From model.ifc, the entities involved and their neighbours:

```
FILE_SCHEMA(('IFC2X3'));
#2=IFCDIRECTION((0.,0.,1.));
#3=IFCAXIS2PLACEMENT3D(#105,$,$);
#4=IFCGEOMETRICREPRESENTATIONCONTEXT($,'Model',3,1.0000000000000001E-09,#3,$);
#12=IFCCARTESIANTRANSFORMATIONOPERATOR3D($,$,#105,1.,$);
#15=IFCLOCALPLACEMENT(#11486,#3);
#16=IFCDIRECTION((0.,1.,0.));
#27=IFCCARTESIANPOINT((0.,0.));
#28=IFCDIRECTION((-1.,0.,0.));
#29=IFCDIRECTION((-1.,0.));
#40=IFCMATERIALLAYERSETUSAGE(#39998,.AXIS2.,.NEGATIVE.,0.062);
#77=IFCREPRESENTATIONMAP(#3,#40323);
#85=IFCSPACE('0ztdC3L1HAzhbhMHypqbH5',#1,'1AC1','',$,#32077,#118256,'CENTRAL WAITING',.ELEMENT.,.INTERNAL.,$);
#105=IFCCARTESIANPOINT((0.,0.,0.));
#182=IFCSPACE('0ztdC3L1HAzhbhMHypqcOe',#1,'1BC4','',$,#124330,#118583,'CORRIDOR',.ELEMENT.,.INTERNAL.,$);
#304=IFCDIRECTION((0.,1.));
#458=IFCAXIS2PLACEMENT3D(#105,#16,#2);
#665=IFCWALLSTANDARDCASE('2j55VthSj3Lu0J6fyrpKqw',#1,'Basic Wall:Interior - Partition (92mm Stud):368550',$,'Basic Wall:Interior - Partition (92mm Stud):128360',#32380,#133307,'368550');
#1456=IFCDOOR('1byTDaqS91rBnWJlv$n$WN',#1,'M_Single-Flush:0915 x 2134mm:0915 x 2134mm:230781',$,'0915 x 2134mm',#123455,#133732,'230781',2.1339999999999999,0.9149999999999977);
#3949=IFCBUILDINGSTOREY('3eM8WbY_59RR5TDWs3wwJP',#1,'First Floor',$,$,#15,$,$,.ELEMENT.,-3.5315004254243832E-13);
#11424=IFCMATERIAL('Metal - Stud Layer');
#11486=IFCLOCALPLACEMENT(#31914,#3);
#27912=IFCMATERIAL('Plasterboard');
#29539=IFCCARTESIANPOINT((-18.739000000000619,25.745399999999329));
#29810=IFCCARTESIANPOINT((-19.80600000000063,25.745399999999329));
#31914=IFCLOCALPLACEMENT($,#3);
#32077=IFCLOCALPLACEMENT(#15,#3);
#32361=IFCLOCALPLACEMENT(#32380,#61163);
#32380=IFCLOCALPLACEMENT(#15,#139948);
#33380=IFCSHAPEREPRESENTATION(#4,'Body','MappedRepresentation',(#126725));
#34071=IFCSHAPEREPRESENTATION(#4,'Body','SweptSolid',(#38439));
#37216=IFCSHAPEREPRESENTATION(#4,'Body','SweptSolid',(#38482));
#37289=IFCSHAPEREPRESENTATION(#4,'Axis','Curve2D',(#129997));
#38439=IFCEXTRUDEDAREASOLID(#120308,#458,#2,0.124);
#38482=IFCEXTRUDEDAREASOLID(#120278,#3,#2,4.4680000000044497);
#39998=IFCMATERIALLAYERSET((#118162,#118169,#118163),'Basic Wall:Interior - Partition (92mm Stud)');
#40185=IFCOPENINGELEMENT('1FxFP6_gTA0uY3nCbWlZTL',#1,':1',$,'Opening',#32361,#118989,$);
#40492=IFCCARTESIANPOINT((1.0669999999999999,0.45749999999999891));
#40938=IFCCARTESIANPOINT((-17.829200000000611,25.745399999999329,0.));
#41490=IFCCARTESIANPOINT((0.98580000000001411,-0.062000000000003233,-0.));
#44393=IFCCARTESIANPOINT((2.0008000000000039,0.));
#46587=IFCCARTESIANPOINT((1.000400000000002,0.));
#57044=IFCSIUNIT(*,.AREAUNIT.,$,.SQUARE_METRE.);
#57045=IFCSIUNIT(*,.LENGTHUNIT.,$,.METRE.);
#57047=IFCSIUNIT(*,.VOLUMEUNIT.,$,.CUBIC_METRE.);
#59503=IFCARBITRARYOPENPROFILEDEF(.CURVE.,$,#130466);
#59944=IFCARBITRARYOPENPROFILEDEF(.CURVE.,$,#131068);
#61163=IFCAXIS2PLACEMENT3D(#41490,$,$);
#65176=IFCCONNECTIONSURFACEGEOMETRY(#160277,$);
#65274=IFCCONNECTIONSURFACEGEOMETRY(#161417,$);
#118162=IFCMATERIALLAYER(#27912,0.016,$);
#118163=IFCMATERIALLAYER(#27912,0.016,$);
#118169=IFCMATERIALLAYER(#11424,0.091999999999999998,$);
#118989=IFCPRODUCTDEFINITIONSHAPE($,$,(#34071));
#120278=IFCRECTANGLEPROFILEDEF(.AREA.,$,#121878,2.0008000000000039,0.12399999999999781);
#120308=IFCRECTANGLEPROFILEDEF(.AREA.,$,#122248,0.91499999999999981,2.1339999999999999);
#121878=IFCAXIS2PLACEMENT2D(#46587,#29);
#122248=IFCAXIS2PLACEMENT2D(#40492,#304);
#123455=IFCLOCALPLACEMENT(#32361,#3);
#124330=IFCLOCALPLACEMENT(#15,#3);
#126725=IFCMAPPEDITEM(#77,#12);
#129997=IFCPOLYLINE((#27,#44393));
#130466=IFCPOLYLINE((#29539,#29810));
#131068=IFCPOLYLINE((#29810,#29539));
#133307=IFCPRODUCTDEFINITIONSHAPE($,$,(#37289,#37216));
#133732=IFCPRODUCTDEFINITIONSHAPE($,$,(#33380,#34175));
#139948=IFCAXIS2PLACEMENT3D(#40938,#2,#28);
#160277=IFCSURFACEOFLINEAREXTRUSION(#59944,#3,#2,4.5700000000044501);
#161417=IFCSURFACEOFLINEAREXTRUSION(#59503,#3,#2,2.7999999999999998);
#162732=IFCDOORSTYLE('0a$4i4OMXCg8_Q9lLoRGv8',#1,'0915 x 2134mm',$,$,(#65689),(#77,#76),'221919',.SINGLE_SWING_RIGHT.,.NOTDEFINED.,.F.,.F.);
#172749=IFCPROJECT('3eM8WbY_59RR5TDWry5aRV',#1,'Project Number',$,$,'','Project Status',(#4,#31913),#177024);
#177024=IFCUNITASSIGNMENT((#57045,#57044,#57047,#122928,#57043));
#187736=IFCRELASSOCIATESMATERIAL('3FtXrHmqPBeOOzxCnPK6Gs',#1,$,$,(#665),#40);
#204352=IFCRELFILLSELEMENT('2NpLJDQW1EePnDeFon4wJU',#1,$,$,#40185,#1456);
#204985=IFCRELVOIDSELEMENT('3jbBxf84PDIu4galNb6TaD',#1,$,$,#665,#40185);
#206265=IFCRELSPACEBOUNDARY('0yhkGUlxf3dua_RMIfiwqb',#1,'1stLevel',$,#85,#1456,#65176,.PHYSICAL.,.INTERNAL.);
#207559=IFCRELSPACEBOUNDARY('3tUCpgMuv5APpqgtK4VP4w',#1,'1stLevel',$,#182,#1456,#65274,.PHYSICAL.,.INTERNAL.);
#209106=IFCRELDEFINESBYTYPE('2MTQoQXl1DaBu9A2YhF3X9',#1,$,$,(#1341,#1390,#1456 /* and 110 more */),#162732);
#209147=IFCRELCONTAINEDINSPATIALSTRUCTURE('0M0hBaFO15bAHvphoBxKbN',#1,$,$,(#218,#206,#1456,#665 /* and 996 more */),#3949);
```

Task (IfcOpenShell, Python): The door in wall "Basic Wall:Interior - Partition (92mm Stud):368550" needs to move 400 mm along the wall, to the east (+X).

```python
import numpy as np
import ifcopenshell
import ifcopenshell.api.geometry
import ifcopenshell.util.placement
import ifcopenshell.util.unit

model = ifcopenshell.open("model.ifc")
unit_scale = ifcopenshell.util.unit.calculate_unit_scale(model)

door = model.by_guid("1byTDaqS91rBnWJlv$n$WN")
opening = door.FillsVoids[0].RelatingOpeningElement
wall = opening.VoidsElements[0].RelatingBuildingElement

wall_matrix = ifcopenshell.util.placement.get_local_placement(wall.ObjectPlacement)
shift = wall_matrix[:3, 0] * -0.4 / unit_scale
before = ifcopenshell.util.placement.get_local_placement(door.ObjectPlacement)[:3, 3].copy()

# The door is placed relative to its opening, so it follows when the opening moves.
matrix = ifcopenshell.util.placement.get_local_placement(opening.ObjectPlacement)
matrix[:3, 3] += shift
ifcopenshell.api.geometry.edit_object_placement(
    model, product=opening, matrix=matrix, is_si=False, should_transform_children=True
)

# Space boundary surfaces are stored in each space's coordinates; move them too.
for rel in door.ProvidesBoundaries:
    if not rel.ConnectionGeometry:
        continue
    surface = rel.ConnectionGeometry.SurfaceOnRelatingElement
    space_matrix = ifcopenshell.util.placement.get_local_placement(rel.RelatingSpace.ObjectPlacement)
    point = np.array(surface.Position.Location.Coordinates) + space_matrix[:3, :3].T @ shift
    surface.Position = model.createIfcAxis2Placement3D(
        model.createIfcCartesianPoint(point.tolist()), surface.Position.Axis, surface.Position.RefDirection
    )

after = ifcopenshell.util.placement.get_local_placement(door.ObjectPlacement)[:3, 3]
print("door moved by", (after - before).round(3) + 0.0)

model.write("model-out.ifc")
```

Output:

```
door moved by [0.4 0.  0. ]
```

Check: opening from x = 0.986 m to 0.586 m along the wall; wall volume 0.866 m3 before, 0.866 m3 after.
